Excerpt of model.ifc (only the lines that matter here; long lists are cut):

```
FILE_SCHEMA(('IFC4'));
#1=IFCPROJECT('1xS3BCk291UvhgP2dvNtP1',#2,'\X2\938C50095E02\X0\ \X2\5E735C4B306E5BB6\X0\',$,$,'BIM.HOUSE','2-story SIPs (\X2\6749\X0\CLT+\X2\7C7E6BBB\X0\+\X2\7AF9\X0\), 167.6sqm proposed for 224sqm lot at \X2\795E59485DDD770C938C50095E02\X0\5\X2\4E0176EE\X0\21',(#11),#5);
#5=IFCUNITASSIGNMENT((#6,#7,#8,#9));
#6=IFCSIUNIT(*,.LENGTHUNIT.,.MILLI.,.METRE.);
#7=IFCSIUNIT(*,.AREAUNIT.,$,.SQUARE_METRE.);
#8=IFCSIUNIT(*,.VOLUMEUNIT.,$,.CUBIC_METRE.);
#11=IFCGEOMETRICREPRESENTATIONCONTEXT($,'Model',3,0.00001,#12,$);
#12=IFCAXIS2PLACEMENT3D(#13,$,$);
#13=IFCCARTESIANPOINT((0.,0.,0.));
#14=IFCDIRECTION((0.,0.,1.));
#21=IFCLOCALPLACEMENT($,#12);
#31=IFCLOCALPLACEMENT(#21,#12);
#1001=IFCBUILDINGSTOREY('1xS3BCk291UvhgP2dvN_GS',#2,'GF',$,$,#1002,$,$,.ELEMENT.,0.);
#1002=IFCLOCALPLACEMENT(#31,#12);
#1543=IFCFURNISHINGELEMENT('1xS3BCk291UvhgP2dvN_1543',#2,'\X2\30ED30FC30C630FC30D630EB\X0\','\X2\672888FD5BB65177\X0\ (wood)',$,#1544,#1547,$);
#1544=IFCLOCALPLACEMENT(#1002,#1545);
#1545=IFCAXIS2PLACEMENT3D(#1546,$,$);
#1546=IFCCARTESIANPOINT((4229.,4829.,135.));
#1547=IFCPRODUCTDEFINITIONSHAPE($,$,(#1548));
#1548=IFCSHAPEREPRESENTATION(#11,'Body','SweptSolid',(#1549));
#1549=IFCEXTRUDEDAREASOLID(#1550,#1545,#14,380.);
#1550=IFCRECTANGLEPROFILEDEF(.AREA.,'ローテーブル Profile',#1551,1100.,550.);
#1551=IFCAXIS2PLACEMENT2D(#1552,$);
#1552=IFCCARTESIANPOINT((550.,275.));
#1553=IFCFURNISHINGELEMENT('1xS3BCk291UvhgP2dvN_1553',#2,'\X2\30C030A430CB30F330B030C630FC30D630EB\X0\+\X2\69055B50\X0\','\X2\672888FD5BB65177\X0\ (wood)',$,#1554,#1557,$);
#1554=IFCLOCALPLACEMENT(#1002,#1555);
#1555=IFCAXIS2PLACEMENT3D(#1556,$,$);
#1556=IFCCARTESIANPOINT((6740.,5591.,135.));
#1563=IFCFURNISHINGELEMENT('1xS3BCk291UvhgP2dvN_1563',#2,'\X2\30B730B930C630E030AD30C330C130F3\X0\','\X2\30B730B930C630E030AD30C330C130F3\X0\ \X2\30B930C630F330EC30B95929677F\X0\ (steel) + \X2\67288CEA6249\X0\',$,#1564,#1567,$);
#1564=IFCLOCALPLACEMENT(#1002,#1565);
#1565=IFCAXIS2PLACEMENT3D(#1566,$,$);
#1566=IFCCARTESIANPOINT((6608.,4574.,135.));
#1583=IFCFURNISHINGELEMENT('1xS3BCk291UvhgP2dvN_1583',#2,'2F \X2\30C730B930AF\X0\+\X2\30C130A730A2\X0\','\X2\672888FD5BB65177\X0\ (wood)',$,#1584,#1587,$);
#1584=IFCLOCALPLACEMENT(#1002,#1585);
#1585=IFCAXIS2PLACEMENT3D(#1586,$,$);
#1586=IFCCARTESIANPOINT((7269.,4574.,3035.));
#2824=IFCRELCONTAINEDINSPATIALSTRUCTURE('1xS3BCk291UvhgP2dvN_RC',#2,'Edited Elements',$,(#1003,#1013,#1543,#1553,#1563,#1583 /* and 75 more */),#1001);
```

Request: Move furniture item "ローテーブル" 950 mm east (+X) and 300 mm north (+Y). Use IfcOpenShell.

```python
import ifcopenshell
import ifcopenshell.api.geometry
import ifcopenshell.util.placement

model = ifcopenshell.open("model.ifc")

item = model.by_id(1543)
matrix = ifcopenshell.util.placement.get_local_placement(item.ObjectPlacement)
matrix[0, 3] += 950.0
matrix[1, 3] += 300.0
ifcopenshell.api.geometry.edit_object_placement(model, product=item, matrix=matrix, is_si=False)

print(ifcopenshell.util.placement.get_local_placement(item.ObjectPlacement).round(3) + 0.0)

model.write("model_updated.ifc")
```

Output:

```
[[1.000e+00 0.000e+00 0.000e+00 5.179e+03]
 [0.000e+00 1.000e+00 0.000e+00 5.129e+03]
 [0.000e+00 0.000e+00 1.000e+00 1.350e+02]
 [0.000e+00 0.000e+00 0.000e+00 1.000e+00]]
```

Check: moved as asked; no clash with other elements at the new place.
